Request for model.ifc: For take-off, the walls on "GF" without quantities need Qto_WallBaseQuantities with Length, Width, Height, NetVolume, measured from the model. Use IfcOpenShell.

First a look at what the model holds.

```python
import ifcopenshell
import ifcopenshell.util.element
import ifcopenshell.util.unit

model = ifcopenshell.open("model.ifc")
print(model.schema)
for unit_type in ("LENGTHUNIT", "AREAUNIT", "VOLUMEUNIT"):
    print(unit_type, ifcopenshell.util.unit.calculate_unit_scale(model, unit_type))
storey = next(s for s in model.by_type("IfcBuildingStorey") if s.Name == "GF")
walls = [e for e in ifcopenshell.util.element.get_decomposition(storey) if e.is_a("IfcWall")]
for e in sorted(walls, key=lambda e: e.id()):
    print(e.id(), e.is_a(), e.Name, list(ifcopenshell.util.element.get_psets(e, qtos_only=True)), sep=" | ")
```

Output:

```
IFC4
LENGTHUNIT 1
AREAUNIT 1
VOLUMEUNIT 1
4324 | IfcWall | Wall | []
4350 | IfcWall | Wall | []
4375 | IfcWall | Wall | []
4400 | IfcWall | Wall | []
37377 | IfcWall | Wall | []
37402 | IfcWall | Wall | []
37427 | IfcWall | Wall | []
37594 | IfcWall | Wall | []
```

```python
import ifcopenshell
import ifcopenshell.api.pset
import ifcopenshell.geom
import ifcopenshell.util.element
import ifcopenshell.util.shape
import ifcopenshell.util.unit

model = ifcopenshell.open("model.ifc")
unit_scale = ifcopenshell.util.unit.calculate_unit_scale(model)
volume_scale = ifcopenshell.util.unit.calculate_unit_scale(model, "VOLUMEUNIT")
settings = ifcopenshell.geom.settings()

storey = next(s for s in model.by_type("IfcBuildingStorey") if s.Name == "GF")
walls = [e for e in ifcopenshell.util.element.get_decomposition(storey) if e.is_a("IfcWall")]

for e in sorted(walls, key=lambda e: e.id()):
    if ifcopenshell.util.element.get_psets(e, qtos_only=True, should_inherit=False):
        continue
    # Geometry comes back in metres, in the element's own axes.
    shape = ifcopenshell.geom.create_shape(settings, e)
    values = {
        "Length": ifcopenshell.util.shape.get_x(shape.geometry) / unit_scale,
        "Width": ifcopenshell.util.shape.get_y(shape.geometry) / unit_scale,
        "Height": ifcopenshell.util.shape.get_z(shape.geometry) / unit_scale,
        "NetVolume": ifcopenshell.util.shape.get_volume(shape.geometry) / volume_scale,
    }
    qto = ifcopenshell.api.pset.add_qto(model, product=e, name="Qto_WallBaseQuantities")
    ifcopenshell.api.pset.edit_qto(model, qto=qto, properties=values)
    print(e.id(), {k: round(v, 3) for k, v in values.items()})

model.write("model_v2.ifc")
```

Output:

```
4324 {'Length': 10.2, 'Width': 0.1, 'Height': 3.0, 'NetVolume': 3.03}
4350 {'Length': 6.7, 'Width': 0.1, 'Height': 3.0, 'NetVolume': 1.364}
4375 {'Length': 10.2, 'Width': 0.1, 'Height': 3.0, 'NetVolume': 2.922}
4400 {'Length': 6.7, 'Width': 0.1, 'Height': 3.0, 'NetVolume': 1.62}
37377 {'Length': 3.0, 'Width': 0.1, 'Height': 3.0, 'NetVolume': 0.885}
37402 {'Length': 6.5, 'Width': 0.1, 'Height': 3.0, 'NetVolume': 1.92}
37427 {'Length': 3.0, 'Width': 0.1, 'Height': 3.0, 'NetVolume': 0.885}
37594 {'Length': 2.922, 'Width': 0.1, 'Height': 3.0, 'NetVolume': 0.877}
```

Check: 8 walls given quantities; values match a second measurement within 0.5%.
